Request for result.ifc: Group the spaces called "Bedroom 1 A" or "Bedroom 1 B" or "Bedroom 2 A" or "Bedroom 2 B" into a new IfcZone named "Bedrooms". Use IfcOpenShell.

First a look at what the model holds.

```python
import ifcopenshell

model = ifcopenshell.open("result.ifc")
print(model.schema)
seen = {}
for space in model.by_type("IfcSpace"):
    seen[space.Name] = seen.get(space.Name, 0) + 1
for name, count in sorted(seen.items(), key=str):
    print(count, "x", name)
print("zones:", [z.Name for z in model.by_type("IfcZone")][:20])
```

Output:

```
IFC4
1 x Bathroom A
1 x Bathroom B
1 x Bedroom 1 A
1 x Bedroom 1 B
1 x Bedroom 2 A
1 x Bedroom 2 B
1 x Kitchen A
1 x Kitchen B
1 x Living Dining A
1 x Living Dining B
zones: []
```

```python
import ifcopenshell
import ifcopenshell.api.group
import ifcopenshell.api.root

model = ifcopenshell.open("result.ifc")

names = {"Bedroom 1 A", "Bedroom 1 B", "Bedroom 2 A", "Bedroom 2 B"}
spaces = [s for s in model.by_type("IfcSpace") if s.Name in names]

zone = ifcopenshell.api.root.create_entity(model, ifc_class="IfcZone", name="Bedrooms")
ifcopenshell.api.group.assign_group(model, products=spaces, group=zone)
print(len(spaces), "spaces in", zone.Name)

model.write("result_v2.ifc")
```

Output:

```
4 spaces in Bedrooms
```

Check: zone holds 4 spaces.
